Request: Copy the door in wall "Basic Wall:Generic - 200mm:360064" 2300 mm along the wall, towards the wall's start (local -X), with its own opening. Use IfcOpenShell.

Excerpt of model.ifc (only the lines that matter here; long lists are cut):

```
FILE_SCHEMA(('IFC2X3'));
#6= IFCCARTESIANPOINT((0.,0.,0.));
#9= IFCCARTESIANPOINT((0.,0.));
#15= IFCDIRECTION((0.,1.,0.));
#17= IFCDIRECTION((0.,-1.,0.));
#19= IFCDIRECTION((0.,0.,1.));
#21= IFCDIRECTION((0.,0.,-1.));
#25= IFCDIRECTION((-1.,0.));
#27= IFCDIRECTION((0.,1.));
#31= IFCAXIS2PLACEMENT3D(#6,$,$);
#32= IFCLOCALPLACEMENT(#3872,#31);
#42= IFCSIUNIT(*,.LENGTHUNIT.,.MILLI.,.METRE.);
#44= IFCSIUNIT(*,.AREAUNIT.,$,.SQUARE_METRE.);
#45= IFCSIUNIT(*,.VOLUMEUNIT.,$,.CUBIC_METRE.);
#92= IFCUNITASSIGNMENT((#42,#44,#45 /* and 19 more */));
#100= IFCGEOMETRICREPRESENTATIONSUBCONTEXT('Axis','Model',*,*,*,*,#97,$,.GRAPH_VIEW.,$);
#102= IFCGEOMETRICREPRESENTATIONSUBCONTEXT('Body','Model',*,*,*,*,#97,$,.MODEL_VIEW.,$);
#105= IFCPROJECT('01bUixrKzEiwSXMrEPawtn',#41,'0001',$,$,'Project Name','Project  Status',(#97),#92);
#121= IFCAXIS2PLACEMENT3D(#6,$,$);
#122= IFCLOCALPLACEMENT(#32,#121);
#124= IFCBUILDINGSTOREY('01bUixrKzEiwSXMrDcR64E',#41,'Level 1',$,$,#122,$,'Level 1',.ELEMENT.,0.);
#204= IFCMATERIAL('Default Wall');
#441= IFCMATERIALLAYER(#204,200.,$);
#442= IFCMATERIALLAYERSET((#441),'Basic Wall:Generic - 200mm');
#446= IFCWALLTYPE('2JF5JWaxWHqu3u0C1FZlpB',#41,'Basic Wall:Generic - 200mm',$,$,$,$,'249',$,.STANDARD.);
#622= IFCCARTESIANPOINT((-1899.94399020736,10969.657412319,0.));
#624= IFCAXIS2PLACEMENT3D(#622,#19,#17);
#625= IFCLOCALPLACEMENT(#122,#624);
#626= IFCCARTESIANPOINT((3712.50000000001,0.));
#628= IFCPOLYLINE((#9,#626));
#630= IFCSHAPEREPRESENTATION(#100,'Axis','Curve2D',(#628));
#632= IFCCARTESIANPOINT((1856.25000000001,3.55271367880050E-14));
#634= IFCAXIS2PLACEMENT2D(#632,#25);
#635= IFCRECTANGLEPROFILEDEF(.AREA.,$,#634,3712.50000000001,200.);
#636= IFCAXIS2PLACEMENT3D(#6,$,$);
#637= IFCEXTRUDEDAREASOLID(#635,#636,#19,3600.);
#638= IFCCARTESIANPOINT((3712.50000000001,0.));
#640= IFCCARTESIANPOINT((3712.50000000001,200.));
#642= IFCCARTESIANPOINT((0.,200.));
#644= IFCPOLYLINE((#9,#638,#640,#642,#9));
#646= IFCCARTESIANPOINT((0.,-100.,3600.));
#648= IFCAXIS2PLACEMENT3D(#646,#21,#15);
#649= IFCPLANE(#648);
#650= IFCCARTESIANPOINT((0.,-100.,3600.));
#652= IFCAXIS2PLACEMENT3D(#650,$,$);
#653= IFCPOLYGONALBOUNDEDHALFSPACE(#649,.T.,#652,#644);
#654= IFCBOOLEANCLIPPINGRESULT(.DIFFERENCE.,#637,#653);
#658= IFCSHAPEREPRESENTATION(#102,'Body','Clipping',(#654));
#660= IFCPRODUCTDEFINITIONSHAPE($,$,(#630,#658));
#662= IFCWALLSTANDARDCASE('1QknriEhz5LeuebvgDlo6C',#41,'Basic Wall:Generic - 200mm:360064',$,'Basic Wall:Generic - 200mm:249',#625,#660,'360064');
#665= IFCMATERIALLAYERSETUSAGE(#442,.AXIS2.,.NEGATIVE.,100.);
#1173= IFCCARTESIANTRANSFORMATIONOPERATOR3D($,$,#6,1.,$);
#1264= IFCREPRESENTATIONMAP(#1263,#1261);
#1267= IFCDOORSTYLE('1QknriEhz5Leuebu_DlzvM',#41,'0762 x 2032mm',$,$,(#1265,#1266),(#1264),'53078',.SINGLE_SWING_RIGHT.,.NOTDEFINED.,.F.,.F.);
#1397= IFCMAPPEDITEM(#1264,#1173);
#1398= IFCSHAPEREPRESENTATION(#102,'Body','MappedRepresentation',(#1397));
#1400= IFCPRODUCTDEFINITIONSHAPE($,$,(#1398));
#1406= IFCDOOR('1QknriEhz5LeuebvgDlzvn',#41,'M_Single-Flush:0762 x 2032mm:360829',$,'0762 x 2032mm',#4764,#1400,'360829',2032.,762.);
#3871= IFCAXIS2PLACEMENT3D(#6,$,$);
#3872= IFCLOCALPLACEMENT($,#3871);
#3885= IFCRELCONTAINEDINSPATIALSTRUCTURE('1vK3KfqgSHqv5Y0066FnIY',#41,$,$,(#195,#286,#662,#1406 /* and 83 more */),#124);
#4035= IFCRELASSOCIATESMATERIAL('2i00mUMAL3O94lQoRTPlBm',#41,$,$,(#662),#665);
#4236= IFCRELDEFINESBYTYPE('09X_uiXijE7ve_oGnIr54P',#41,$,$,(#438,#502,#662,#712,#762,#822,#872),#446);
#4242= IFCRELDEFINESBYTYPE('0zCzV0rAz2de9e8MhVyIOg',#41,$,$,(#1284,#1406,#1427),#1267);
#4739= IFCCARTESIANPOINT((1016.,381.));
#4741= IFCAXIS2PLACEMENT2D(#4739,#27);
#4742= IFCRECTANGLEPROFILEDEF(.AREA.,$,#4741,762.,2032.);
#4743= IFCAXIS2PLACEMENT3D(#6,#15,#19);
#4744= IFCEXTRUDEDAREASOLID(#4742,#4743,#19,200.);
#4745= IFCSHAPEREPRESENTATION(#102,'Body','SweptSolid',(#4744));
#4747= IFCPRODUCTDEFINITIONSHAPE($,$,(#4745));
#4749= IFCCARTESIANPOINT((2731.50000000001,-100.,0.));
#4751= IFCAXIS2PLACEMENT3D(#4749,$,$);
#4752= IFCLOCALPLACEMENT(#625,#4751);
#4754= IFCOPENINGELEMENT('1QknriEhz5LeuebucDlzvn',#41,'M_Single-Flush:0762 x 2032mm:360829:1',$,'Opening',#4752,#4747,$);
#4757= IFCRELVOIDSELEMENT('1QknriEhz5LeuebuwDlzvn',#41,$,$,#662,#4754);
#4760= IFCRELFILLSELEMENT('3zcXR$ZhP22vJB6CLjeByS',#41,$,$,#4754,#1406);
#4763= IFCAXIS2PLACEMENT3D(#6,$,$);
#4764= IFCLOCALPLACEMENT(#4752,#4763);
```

```python
import ifcopenshell
import ifcopenshell.api.feature
import ifcopenshell.api.geometry
import ifcopenshell.api.root
import ifcopenshell.geom
import ifcopenshell.util.element
import ifcopenshell.util.placement
import ifcopenshell.util.shape

model = ifcopenshell.open("model.ifc")
settings = ifcopenshell.geom.settings()


def volume(element):
    """Net volume in cubic metres, openings subtracted."""
    shape = ifcopenshell.geom.create_shape(settings, element)
    return ifcopenshell.util.shape.get_volume(shape.geometry)


def reuse_history(source, copy):
    """copy_class also copies each property set's owner history, people and application; keep the originals."""
    for rel in copy.IsDefinedBy:
        if rel.is_a("IfcRelDefinesByProperties") and (history := rel.RelatingPropertyDefinition.OwnerHistory):
            rel.RelatingPropertyDefinition.OwnerHistory = source.OwnerHistory
            ifcopenshell.util.element.remove_deep2(model, history)


door = model.by_id(1406)
opening = door.FillsVoids[0].RelatingOpeningElement
wall = opening.VoidsElements[0].RelatingBuildingElement
before = volume(wall)
shift = ifcopenshell.util.placement.get_local_placement(wall.ObjectPlacement)[:3, 0] * -2300.0

# copy_class copies the void relationship, type, container and properties, but no geometry.
new_opening = ifcopenshell.api.root.copy_class(model, product=opening)
new_opening.Representation = ifcopenshell.util.element.copy_deep(
    model, opening.Representation, exclude=["IfcGeometricRepresentationContext", "IfcRepresentationMap"]
)
new_opening.Name = "M_Single-Flush:0762 x 2032mm"
new_door = ifcopenshell.api.root.copy_class(model, product=door)
new_door.Representation = ifcopenshell.util.element.copy_deep(
    model, door.Representation, exclude=["IfcGeometricRepresentationContext", "IfcRepresentationMap"]
)
new_door.Name = "M_Single-Flush:0762 x 2032mm"
new_door.Tag = None
reuse_history(door, new_door)
fills = ifcopenshell.api.feature.add_filling(model, opening=new_opening, element=new_door)
fills.OwnerHistory = new_door.OwnerHistory  # required in IFC2X3

for old, new in ((opening, new_opening), (door, new_door)):
    matrix = ifcopenshell.util.placement.get_local_placement(old.ObjectPlacement)
    matrix[:3, 3] += shift
    ifcopenshell.api.geometry.edit_object_placement(model, product=new, matrix=matrix, is_si=False)

after = volume(wall)

print(f"wall volume {before:.3f} -> {after:.3f} m3")

model.write("model_v2.ifc")
```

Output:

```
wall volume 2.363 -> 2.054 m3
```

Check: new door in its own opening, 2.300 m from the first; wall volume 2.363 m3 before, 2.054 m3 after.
